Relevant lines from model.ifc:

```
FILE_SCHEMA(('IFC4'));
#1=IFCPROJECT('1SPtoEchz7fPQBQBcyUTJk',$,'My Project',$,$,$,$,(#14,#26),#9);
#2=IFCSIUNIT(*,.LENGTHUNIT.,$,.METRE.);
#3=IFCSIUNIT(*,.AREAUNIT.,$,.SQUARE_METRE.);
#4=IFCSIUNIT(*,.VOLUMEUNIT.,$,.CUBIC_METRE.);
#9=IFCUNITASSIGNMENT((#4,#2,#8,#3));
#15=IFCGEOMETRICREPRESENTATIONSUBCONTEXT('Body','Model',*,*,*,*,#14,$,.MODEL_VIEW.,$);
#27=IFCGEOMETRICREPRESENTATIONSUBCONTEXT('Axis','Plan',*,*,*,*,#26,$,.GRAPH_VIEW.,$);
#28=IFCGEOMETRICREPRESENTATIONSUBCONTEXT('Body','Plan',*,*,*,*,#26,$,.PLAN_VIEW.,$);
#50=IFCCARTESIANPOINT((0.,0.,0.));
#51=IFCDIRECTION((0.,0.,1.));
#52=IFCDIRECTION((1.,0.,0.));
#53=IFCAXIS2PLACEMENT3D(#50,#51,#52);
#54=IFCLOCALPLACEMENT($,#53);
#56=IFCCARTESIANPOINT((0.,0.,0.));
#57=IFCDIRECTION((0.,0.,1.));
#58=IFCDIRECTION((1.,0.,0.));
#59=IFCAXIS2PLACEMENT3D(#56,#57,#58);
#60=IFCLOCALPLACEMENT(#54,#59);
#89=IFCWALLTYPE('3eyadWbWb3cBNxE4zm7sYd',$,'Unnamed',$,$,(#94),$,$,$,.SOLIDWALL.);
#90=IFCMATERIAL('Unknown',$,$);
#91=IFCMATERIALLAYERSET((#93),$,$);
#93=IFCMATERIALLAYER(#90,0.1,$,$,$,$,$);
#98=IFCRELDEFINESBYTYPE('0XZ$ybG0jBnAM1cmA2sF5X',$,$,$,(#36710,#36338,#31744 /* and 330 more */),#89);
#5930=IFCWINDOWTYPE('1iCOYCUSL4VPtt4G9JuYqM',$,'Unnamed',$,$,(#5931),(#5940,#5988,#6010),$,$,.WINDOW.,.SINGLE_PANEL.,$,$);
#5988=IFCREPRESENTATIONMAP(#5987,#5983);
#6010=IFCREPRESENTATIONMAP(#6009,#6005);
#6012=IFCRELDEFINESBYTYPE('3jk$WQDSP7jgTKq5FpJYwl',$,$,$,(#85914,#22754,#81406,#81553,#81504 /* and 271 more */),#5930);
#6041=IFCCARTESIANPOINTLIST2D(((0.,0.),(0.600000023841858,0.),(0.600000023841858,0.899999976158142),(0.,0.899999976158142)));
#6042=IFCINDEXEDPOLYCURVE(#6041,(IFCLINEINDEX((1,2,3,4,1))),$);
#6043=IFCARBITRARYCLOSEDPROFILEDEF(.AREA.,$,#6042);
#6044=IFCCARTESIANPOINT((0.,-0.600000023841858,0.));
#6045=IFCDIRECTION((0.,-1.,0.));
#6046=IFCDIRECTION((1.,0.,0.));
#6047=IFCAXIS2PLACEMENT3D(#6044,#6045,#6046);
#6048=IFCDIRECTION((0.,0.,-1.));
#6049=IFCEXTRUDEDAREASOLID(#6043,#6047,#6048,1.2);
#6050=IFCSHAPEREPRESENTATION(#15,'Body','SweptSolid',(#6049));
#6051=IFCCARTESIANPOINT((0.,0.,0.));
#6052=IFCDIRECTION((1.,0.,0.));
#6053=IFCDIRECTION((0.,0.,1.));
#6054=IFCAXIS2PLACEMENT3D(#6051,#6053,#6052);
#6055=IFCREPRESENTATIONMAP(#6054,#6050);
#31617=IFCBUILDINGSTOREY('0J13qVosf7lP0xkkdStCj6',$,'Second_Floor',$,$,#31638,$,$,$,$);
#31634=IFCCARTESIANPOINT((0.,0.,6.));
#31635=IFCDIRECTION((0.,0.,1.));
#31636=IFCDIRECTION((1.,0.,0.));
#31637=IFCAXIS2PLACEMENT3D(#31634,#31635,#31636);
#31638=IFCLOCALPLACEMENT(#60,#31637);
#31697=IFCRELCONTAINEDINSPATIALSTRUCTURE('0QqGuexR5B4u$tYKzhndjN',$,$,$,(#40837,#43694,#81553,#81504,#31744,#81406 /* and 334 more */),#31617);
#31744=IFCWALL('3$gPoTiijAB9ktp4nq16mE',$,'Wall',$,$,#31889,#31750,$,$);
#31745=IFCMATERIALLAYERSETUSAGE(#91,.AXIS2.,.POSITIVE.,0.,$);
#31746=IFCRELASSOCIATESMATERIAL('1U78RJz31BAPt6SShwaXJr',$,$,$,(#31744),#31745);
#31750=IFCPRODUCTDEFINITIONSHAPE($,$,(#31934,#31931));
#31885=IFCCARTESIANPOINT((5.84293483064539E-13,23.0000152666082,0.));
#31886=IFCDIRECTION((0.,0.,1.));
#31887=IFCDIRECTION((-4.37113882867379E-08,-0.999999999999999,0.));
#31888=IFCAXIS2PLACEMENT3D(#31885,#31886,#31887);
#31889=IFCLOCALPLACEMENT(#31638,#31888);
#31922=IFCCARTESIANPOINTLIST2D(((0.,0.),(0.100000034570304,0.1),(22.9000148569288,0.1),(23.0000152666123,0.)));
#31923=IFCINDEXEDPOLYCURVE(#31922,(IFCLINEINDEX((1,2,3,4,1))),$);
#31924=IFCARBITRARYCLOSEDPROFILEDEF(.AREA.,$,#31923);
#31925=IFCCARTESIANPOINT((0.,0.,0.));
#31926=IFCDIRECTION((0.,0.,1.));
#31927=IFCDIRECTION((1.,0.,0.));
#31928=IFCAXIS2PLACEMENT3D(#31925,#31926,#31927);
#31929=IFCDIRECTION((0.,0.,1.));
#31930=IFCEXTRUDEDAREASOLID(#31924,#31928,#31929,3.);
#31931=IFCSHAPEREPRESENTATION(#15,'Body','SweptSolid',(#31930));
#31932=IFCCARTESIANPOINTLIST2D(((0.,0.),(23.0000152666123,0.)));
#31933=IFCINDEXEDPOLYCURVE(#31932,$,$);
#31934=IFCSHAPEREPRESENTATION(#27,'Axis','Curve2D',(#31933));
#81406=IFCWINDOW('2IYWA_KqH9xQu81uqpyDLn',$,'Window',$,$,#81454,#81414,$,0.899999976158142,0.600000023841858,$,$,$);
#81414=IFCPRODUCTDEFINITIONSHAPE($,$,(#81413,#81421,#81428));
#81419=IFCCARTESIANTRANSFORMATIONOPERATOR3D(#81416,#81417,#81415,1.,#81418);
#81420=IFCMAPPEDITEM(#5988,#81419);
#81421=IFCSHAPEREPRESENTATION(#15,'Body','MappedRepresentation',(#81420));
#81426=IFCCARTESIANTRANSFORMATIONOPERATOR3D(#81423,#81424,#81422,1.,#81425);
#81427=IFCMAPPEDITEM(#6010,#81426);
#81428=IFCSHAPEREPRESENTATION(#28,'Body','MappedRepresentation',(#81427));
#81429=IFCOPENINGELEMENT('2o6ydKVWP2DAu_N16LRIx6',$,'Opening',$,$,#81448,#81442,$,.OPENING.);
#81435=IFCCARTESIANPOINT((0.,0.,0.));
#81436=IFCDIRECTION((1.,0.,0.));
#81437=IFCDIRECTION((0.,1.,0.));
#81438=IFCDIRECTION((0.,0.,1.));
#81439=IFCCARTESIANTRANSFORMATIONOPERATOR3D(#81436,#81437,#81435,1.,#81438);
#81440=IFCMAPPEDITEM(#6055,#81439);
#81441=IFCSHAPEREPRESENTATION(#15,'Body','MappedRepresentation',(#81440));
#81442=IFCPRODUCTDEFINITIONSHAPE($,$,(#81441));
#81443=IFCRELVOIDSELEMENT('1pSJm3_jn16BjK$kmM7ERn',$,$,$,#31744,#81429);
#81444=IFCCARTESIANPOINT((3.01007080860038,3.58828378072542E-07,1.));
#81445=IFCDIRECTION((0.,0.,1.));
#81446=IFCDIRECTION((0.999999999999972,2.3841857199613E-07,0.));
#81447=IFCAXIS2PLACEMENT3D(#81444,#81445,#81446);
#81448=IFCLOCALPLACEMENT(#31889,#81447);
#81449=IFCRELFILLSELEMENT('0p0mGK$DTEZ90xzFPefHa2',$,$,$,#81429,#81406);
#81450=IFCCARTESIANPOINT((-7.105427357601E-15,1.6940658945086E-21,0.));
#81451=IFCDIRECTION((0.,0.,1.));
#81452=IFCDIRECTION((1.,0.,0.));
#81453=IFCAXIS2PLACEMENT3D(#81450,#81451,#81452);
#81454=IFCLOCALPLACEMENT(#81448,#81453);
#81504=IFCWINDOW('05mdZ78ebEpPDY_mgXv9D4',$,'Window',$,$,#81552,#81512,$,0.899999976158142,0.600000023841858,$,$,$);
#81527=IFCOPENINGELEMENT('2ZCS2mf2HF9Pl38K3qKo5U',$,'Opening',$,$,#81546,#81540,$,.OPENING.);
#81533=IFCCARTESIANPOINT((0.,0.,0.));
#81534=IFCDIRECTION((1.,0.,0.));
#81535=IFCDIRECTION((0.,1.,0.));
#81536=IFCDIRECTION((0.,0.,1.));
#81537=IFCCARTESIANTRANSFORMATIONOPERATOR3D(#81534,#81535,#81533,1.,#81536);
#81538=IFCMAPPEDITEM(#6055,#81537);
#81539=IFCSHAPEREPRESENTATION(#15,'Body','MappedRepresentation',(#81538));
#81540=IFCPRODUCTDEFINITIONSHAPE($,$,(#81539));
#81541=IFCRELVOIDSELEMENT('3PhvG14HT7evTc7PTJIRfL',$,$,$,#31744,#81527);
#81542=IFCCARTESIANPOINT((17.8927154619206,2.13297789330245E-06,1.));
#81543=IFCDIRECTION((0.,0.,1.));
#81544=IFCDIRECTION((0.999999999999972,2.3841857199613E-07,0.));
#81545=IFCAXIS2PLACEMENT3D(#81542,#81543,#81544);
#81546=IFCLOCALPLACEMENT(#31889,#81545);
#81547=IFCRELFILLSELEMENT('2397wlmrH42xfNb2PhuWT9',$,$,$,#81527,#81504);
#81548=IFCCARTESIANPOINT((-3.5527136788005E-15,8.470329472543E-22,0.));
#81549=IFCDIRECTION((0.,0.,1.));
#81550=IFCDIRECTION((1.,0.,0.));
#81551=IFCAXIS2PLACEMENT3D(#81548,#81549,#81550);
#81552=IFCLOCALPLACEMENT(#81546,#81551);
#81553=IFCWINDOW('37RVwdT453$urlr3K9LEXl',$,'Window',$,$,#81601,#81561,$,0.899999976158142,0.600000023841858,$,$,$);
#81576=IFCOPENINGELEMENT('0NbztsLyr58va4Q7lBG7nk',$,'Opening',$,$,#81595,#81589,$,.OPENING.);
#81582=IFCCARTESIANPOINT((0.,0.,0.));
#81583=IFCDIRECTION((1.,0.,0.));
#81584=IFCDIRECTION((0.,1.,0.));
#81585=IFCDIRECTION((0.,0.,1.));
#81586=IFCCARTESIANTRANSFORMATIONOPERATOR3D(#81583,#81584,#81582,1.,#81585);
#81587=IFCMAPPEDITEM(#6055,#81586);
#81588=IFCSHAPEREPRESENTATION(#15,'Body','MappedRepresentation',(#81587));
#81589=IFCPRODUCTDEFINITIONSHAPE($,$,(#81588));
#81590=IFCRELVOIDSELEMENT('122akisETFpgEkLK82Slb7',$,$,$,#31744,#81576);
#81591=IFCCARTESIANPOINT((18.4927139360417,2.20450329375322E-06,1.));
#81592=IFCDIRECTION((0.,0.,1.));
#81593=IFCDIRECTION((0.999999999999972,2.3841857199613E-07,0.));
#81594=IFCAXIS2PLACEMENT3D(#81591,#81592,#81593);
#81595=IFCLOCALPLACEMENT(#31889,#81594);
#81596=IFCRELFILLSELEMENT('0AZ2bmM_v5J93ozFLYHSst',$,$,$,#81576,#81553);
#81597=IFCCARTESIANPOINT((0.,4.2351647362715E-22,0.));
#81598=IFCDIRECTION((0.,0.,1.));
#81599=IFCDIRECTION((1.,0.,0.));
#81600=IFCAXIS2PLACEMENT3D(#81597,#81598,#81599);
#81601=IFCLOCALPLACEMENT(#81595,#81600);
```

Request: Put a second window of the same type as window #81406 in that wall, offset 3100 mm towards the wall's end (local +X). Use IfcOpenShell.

```python
import ifcopenshell
import ifcopenshell.api.feature
import ifcopenshell.api.geometry
import ifcopenshell.api.root
import ifcopenshell.geom
import ifcopenshell.util.element
import ifcopenshell.util.placement
import ifcopenshell.util.shape
import ifcopenshell.util.unit

model = ifcopenshell.open("model.ifc")
unit_scale = ifcopenshell.util.unit.calculate_unit_scale(model)
settings = ifcopenshell.geom.settings()


def volume(element):
    """Net volume in cubic metres, openings subtracted."""
    shape = ifcopenshell.geom.create_shape(settings, element)
    return ifcopenshell.util.shape.get_volume(shape.geometry)


window = model.by_guid("2IYWA_KqH9xQu81uqpyDLn")
opening = window.FillsVoids[0].RelatingOpeningElement
wall = opening.VoidsElements[0].RelatingBuildingElement
before = volume(wall)
shift = ifcopenshell.util.placement.get_local_placement(wall.ObjectPlacement)[:3, 0] * 3.1 / unit_scale

# copy_class copies the void relationship, type, container and properties, but no geometry.
new_opening = ifcopenshell.api.root.copy_class(model, product=opening)
new_opening.Representation = ifcopenshell.util.element.copy_deep(
    model, opening.Representation, exclude=["IfcGeometricRepresentationContext", "IfcRepresentationMap"]
)
new_window = ifcopenshell.api.root.copy_class(model, product=window)
new_window.Representation = ifcopenshell.util.element.copy_deep(
    model, window.Representation, exclude=["IfcGeometricRepresentationContext", "IfcRepresentationMap"]
)
ifcopenshell.api.feature.add_filling(model, opening=new_opening, element=new_window)

for old, new in ((opening, new_opening), (window, new_window)):
    matrix = ifcopenshell.util.placement.get_local_placement(old.ObjectPlacement)
    matrix[:3, 3] += shift
    ifcopenshell.api.geometry.edit_object_placement(model, product=new, matrix=matrix, is_si=False)

after = volume(wall)

print(f"wall volume {before:.3f} -> {after:.3f} m3")

model.write("model_v2.ifc")
```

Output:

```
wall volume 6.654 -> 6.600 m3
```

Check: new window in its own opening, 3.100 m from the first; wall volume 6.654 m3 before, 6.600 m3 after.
